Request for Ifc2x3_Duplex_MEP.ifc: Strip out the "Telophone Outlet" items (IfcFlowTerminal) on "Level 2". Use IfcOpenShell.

First a look at what the model holds.

```python
import ifcopenshell
import ifcopenshell.util.element

model = ifcopenshell.open("Ifc2x3_Duplex_MEP.ifc")
print(model.schema)
storey = next(s for s in model.by_type("IfcBuildingStorey") if s.Name == "Level 2")
terminals = [e for e in ifcopenshell.util.element.get_decomposition(storey) if e.is_a("IfcFlowTerminal")]
seen = {}
for e in terminals:
    element_type = ifcopenshell.util.element.get_type(e)
    name = element_type.Name if element_type not in (None, e) else None
    seen[name] = seen.get(name, 0) + 1
for name, count in sorted(seen.items(), key=str):
    print(count, "x", name)
```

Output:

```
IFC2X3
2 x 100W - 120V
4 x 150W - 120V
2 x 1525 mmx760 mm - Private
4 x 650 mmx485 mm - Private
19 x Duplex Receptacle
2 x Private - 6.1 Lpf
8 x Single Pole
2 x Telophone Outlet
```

```python
import ifcopenshell
import ifcopenshell.api.root
import ifcopenshell.util.element

model = ifcopenshell.open("Ifc2x3_Duplex_MEP.ifc")

storey = next(s for s in model.by_type("IfcBuildingStorey") if s.Name == "Level 2")
terminals = [e for e in ifcopenshell.util.element.get_decomposition(storey) if e.is_a("IfcFlowTerminal")]
targets = [e for e in terminals if (t := ifcopenshell.util.element.get_type(e)) not in (None, e) and t.Name == "Telophone Outlet"]

for e in targets:
    ifcopenshell.api.root.remove_product(model, product=e)
print(len(targets), "removed")

model.write("Ifc2x3_Duplex_MEP-out.ifc")
```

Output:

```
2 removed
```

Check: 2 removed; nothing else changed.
